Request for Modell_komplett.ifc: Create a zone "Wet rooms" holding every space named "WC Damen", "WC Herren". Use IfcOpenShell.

First a look at what the model holds.

```python
import ifcopenshell

model = ifcopenshell.open("Modell_komplett.ifc")
print(model.schema)
seen = {}
for space in model.by_type("IfcSpace"):
    seen[space.LongName] = seen.get(space.LongName, 0) + 1
for name, count in sorted(seen.items(), key=str):
    print(count, "x", name)
print("zones:", [z.Name for z in model.by_type("IfcZone")][:20])
```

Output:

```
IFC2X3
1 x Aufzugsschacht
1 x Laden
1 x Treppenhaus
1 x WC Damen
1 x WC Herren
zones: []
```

```python
import ifcopenshell
import ifcopenshell.api.group
import ifcopenshell.api.root

model = ifcopenshell.open("Modell_komplett.ifc")

names = {"WC Damen", "WC Herren"}
spaces = [s for s in model.by_type("IfcSpace") if s.LongName in names]

zone = ifcopenshell.api.root.create_entity(model, ifc_class="IfcZone", name="Wet rooms")
ifcopenshell.api.group.assign_group(model, products=spaces, group=zone)
print(len(spaces), "spaces in", zone.Name)

model.write("Modell_komplett_v2.ifc")
```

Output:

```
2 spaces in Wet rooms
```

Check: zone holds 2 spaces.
